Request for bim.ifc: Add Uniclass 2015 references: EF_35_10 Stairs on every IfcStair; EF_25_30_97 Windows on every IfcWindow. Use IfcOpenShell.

First a look at what the model holds.

```python
import ifcopenshell

model = ifcopenshell.open("bim.ifc")
print(model.schema)
print("classifications:", [c.Name for c in model.by_type("IfcClassification")])
for ifc_class in ("IfcDoor", "IfcRoof", "IfcStair", "IfcWall", "IfcWindow"):
    print(ifc_class, len(model.by_type(ifc_class)))
```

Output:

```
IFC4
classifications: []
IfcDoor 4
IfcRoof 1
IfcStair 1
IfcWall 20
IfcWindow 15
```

```python
import ifcopenshell
import ifcopenshell.api.classification

model = ifcopenshell.open("bim.ifc")

system = ifcopenshell.api.classification.add_classification(model, classification="Uniclass 2015")

codes = {
    "IfcStair": ("EF_35_10", "Stairs"),
    "IfcWindow": ("EF_25_30_97", "Windows"),
}
for ifc_class, (code, name) in codes.items():
    products = model.by_type(ifc_class)
    ifcopenshell.api.classification.add_reference(
        model, products=products, classification=system, identification=code, name=name
    )
    print(code, len(products))

model.write("bim-out.ifc")
```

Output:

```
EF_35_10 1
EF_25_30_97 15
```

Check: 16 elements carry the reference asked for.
